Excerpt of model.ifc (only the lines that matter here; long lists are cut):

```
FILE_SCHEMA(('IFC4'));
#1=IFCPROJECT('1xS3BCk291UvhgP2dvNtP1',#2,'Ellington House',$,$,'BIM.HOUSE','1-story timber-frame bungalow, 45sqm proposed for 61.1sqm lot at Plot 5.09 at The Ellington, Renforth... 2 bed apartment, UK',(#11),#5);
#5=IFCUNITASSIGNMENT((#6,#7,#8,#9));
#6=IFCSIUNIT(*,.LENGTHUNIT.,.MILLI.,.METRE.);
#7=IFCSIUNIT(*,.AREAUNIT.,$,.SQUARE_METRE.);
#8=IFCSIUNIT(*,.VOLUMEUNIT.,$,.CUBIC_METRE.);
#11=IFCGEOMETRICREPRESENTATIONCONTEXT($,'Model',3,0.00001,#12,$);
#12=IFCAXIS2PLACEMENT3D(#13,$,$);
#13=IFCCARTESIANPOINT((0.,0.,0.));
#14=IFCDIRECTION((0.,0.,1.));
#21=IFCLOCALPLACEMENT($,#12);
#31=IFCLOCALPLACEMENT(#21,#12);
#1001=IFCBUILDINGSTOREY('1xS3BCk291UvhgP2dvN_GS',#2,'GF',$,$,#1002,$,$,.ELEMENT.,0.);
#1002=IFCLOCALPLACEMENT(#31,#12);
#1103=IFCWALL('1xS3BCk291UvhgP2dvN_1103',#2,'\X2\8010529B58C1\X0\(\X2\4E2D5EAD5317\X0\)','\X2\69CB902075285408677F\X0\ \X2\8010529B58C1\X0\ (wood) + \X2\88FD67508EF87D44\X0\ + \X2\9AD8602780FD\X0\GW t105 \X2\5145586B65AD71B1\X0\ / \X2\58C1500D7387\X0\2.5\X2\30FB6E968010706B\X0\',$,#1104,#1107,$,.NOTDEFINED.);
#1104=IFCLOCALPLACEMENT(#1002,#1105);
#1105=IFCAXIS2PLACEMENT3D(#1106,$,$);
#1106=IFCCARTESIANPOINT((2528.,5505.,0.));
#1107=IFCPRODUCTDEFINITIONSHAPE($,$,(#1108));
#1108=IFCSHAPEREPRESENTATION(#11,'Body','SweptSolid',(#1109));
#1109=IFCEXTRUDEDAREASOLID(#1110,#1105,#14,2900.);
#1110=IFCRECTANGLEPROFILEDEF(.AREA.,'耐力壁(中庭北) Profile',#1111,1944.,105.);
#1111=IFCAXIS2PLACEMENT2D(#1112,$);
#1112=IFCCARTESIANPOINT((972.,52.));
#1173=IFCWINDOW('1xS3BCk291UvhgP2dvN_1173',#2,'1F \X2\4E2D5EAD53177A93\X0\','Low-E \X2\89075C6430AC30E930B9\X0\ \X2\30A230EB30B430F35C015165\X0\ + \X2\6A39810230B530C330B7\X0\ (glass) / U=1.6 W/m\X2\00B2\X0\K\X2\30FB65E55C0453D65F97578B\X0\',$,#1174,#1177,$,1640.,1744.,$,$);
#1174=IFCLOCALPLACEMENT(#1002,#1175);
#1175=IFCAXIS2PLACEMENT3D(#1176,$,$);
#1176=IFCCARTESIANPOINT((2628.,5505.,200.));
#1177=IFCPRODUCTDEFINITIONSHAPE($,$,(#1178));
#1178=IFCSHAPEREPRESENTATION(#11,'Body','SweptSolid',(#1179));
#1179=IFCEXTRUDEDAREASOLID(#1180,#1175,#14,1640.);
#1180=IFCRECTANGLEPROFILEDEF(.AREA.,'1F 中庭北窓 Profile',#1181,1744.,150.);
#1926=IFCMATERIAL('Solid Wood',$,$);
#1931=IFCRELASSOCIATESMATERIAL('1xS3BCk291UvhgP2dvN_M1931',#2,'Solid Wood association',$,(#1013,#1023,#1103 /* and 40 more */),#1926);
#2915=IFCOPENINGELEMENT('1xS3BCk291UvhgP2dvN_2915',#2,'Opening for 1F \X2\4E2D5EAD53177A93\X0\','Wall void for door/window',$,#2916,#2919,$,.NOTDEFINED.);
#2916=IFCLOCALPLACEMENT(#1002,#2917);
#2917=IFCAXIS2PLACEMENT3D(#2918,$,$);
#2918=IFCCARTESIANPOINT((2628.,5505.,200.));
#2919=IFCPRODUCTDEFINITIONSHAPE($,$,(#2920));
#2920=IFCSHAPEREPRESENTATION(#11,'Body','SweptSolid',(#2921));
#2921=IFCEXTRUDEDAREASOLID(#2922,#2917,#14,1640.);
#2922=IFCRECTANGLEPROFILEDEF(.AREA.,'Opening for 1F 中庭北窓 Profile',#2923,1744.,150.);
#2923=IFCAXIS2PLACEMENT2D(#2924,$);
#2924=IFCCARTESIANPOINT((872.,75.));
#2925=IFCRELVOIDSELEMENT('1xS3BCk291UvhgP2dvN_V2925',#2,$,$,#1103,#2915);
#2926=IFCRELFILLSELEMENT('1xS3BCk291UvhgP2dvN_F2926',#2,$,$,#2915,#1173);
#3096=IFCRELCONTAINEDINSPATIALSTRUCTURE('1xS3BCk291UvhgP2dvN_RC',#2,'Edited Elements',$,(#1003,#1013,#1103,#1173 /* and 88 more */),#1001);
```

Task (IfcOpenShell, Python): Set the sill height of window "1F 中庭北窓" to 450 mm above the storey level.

```python
import numpy as np
import ifcopenshell
import ifcopenshell.api.geometry
import ifcopenshell.geom
import ifcopenshell.util.element
import ifcopenshell.util.placement
import ifcopenshell.util.shape
import ifcopenshell.util.unit

model = ifcopenshell.open("model.ifc")
unit_scale = ifcopenshell.util.unit.calculate_unit_scale(model)

window = model.by_id(1173)
opening = window.FillsVoids[0].RelatingOpeningElement
storey = ifcopenshell.util.element.get_container(window, ifc_class="IfcBuildingStorey")
level = ifcopenshell.util.placement.get_local_placement(storey.ObjectPlacement)[2, 3]

# The opening's origin need not be at the sill, so measure its lowest point.
shape = ifcopenshell.geom.create_shape(ifcopenshell.geom.settings(), opening)
bottom = ifcopenshell.util.shape.get_shape_bottom_elevation(shape, shape.geometry) / unit_scale
dz = level + 450.0 - bottom

shift = np.array([0.0, 0.0, dz])
# The window is not placed relative to its opening, so move both.
for product in (opening, window):
    matrix = ifcopenshell.util.placement.get_local_placement(product.ObjectPlacement)
    matrix[:3, 3] += shift
    ifcopenshell.api.geometry.edit_object_placement(model, product=product, matrix=matrix, is_si=False)

print(f"moved by {dz * unit_scale:+.3f} m")

model.write("model_rev.ifc")
```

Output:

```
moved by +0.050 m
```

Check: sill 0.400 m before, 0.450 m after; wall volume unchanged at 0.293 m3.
